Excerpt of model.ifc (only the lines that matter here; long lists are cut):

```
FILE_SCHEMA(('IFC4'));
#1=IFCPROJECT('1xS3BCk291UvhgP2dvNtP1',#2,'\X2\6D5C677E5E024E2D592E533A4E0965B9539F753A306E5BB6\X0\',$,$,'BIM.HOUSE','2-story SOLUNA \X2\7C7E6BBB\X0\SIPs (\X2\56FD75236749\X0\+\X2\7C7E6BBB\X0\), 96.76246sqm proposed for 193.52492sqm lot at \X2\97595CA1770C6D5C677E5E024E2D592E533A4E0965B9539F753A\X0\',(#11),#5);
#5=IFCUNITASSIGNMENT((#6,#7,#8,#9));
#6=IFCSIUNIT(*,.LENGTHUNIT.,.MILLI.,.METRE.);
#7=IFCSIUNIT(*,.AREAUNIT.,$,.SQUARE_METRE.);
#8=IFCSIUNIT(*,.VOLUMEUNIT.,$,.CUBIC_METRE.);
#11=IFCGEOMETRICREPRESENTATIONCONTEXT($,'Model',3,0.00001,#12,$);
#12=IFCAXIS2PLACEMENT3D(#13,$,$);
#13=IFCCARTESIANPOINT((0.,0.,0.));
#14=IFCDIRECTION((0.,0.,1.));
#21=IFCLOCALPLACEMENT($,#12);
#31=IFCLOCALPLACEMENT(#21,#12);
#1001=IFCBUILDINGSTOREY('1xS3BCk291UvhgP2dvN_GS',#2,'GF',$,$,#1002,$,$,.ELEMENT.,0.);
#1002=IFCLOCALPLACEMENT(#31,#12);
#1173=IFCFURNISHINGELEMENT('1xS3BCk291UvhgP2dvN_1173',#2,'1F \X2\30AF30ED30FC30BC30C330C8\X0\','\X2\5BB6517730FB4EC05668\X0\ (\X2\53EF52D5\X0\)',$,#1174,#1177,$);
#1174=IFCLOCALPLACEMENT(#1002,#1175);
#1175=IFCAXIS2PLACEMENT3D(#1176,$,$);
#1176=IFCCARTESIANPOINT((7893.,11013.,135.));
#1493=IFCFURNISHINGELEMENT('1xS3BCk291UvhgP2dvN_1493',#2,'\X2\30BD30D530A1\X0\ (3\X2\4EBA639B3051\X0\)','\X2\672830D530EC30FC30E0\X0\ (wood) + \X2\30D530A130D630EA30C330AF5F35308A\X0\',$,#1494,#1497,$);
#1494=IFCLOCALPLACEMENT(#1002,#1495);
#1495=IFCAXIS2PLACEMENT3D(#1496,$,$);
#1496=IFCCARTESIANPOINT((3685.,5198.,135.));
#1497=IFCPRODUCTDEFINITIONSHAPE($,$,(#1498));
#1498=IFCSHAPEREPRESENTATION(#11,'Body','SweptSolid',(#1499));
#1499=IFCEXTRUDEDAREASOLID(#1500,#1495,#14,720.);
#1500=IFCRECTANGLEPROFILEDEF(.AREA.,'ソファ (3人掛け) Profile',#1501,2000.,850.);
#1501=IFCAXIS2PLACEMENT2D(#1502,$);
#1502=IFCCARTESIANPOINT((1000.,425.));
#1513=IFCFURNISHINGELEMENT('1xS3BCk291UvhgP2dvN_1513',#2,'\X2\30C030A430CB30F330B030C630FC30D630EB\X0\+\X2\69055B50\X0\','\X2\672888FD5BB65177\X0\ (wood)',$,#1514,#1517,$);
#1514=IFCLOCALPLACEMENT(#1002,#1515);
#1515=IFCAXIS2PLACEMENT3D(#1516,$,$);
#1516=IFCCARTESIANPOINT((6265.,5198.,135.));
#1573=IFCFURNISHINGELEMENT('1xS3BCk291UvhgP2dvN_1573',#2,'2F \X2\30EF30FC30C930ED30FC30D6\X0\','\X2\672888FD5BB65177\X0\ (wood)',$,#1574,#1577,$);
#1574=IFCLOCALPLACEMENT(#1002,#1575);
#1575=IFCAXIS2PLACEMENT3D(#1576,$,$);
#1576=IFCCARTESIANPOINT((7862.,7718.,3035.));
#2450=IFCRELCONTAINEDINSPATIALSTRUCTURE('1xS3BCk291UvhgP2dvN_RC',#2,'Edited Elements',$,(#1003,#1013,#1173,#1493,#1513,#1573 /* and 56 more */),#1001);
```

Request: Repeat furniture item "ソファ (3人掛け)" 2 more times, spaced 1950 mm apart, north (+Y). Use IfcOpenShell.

```python
import numpy as np
import ifcopenshell
import ifcopenshell.api.geometry
import ifcopenshell.api.root
import ifcopenshell.util.element
import ifcopenshell.util.placement
import ifcopenshell.util.unit

model = ifcopenshell.open("model.ifc")
unit_scale = ifcopenshell.util.unit.calculate_unit_scale(model)


def reuse_history(source, copy):
    """copy_class also copies each property set's owner history, people and application; keep the originals."""
    for rel in copy.IsDefinedBy:
        if rel.is_a("IfcRelDefinesByProperties") and (history := rel.RelatingPropertyDefinition.OwnerHistory):
            rel.RelatingPropertyDefinition.OwnerHistory = source.OwnerHistory
            ifcopenshell.util.element.remove_deep2(model, history)


source = model.by_guid("1xS3BCk291UvhgP2dvN_1493")
base = ifcopenshell.util.placement.get_local_placement(source.ObjectPlacement)
step = np.array([0.0, 1.0, 0.0]) * 1.95 / unit_scale

for i in range(1, 3):
    copy = ifcopenshell.api.root.copy_class(model, product=source)
    copy.Representation = ifcopenshell.util.element.copy_deep(
        model, source.Representation, exclude=["IfcGeometricRepresentationContext", "IfcRepresentationMap"]
    )
    reuse_history(source, copy)
    matrix = base.copy()
    matrix[:3, 3] += i * step
    print("added at", matrix[:3, 3].round(3) + 0.0)
    ifcopenshell.api.geometry.edit_object_placement(model, product=copy, matrix=matrix, is_si=False)

model.write("model-out.ifc")
```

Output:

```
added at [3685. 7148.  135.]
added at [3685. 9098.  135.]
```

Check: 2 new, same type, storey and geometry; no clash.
